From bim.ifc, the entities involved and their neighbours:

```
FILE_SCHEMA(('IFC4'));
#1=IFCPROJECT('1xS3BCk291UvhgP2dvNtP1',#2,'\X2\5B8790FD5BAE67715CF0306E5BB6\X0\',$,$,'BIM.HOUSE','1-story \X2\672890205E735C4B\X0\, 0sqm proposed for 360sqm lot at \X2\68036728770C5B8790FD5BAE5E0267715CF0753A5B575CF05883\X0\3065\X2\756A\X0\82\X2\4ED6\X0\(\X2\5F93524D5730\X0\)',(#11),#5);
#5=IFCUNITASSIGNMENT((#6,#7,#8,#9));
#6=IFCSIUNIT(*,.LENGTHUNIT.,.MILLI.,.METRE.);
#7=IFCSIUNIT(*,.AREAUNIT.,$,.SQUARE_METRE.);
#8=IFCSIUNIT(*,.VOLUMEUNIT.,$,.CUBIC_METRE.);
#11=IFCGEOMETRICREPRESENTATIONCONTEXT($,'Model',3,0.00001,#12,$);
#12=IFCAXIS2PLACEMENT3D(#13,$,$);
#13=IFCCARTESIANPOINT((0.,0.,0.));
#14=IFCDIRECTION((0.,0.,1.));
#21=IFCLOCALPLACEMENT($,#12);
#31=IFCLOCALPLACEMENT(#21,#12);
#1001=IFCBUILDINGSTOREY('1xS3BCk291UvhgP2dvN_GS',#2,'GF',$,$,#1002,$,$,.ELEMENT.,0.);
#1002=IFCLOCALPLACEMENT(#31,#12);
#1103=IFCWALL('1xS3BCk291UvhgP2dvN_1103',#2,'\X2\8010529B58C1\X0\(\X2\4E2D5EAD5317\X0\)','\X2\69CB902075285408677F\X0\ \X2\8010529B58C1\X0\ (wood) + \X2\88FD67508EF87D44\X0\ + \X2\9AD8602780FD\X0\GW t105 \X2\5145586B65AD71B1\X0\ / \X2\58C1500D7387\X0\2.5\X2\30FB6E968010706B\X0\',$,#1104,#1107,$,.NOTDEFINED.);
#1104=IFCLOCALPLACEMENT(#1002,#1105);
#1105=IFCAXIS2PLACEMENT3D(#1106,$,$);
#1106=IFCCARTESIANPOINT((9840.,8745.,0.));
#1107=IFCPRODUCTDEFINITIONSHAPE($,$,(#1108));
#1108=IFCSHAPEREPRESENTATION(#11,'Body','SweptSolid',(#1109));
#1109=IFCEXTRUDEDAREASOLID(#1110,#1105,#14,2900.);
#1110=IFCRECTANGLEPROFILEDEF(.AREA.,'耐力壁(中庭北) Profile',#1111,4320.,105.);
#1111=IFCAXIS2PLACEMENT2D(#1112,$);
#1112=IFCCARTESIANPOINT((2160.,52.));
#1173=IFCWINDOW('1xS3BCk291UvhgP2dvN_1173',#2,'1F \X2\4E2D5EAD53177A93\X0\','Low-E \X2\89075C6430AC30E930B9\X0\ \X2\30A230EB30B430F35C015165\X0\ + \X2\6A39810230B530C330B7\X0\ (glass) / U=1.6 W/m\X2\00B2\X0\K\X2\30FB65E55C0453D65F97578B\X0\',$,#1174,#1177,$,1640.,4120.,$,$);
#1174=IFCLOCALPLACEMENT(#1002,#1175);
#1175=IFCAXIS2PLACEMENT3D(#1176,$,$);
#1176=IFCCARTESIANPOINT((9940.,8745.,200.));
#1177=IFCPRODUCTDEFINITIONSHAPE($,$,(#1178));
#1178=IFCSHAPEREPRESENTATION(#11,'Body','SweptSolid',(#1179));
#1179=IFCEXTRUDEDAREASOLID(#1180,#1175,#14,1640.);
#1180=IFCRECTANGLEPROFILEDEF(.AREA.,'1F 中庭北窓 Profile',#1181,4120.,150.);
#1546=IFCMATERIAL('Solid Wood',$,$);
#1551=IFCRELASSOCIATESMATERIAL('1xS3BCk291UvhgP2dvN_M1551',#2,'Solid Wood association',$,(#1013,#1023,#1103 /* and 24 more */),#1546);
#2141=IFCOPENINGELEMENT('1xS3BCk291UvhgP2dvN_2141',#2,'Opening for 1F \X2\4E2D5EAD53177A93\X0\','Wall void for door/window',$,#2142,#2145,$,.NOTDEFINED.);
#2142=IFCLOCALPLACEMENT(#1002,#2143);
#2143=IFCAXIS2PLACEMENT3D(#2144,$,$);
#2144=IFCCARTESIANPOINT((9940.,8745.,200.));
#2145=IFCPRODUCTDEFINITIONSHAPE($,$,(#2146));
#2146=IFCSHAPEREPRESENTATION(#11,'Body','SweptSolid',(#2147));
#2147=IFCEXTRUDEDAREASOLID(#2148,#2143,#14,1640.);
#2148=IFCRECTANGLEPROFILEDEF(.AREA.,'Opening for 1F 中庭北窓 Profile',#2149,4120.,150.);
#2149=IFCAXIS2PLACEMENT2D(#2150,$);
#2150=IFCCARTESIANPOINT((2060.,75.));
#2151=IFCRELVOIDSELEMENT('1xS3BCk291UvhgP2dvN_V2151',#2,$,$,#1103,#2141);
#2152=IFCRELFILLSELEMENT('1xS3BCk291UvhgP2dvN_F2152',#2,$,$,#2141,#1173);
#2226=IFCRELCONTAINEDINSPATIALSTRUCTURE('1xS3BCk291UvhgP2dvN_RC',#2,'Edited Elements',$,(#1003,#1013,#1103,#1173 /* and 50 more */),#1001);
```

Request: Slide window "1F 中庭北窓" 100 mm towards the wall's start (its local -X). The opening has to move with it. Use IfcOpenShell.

```python
import ifcopenshell
import ifcopenshell.api.geometry
import ifcopenshell.util.placement
import ifcopenshell.util.unit

model = ifcopenshell.open("bim.ifc")
unit_scale = ifcopenshell.util.unit.calculate_unit_scale(model)

window = model.by_id(1173)
opening = window.FillsVoids[0].RelatingOpeningElement
wall = opening.VoidsElements[0].RelatingBuildingElement

wall_matrix = ifcopenshell.util.placement.get_local_placement(wall.ObjectPlacement)
shift = wall_matrix[:3, 0] * -0.1 / unit_scale
before = ifcopenshell.util.placement.get_local_placement(window.ObjectPlacement)[:3, 3].copy()

# The window is not placed relative to its opening, so move both.
for product in (opening, window):
    matrix = ifcopenshell.util.placement.get_local_placement(product.ObjectPlacement)
    matrix[:3, 3] += shift
    ifcopenshell.api.geometry.edit_object_placement(model, product=product, matrix=matrix, is_si=False)

after = ifcopenshell.util.placement.get_local_placement(window.ObjectPlacement)[:3, 3]
print("window moved by", (after - before).round(3) + 0.0)

model.write("bim_v2.ifc")
```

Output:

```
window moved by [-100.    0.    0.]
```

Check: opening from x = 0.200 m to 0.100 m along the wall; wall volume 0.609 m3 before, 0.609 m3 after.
